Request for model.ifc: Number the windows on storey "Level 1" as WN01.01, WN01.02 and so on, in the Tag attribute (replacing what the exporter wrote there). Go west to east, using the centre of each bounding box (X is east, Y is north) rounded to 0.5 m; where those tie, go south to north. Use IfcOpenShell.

First a look at what the model holds.

```python
import ifcopenshell
import ifcopenshell.util.element
import ifcopenshell.util.placement

model = ifcopenshell.open("model.ifc")
print(model.schema)
storey = next(s for s in model.by_type("IfcBuildingStorey") if s.Name == "Level 1")
windows = [e for e in ifcopenshell.util.element.get_decomposition(storey) if e.is_a("IfcWindow")]
for e in sorted(windows, key=lambda e: e.id()):
    origin = ifcopenshell.util.placement.get_local_placement(e.ObjectPlacement)[:3, 3]
    print(e.id(), e.Tag, e.Name, origin.round(2) + 0.0, sep=" | ")
```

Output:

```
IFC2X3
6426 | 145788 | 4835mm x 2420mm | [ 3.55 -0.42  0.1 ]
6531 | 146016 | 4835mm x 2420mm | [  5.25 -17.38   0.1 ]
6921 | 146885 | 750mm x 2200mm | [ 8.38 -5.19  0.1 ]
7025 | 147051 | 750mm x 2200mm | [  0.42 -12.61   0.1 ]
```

```python
import ifcopenshell
import ifcopenshell.geom
import ifcopenshell.util.element
import ifcopenshell.util.shape

model = ifcopenshell.open("model.ifc")
settings = ifcopenshell.geom.settings()
settings.set("use-world-coords", True)


def centre(element):
    shape = ifcopenshell.geom.create_shape(settings, element)
    return ifcopenshell.util.shape.get_bbox_centroid(shape.geometry)


storey = next(s for s in model.by_type("IfcBuildingStorey") if s.Name == "Level 1")
windows = [e for e in ifcopenshell.util.element.get_decomposition(storey) if e.is_a("IfcWindow")]

# Insertion points can sit at a corner or the storey origin, so sort by the geometry (in metres).
centres = {e: centre(e) for e in windows}
windows.sort(key=lambda e: (round(centres[e][0] / 0.5), centres[e][1]))

for i, e in enumerate(windows, start=1):
    number = f"WN01.{i:02d}"
    e.Tag = number
    print(e.id(), number)

model.write("model_rev.ifc")
```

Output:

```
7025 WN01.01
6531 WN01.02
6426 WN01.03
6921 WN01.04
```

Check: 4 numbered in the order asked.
